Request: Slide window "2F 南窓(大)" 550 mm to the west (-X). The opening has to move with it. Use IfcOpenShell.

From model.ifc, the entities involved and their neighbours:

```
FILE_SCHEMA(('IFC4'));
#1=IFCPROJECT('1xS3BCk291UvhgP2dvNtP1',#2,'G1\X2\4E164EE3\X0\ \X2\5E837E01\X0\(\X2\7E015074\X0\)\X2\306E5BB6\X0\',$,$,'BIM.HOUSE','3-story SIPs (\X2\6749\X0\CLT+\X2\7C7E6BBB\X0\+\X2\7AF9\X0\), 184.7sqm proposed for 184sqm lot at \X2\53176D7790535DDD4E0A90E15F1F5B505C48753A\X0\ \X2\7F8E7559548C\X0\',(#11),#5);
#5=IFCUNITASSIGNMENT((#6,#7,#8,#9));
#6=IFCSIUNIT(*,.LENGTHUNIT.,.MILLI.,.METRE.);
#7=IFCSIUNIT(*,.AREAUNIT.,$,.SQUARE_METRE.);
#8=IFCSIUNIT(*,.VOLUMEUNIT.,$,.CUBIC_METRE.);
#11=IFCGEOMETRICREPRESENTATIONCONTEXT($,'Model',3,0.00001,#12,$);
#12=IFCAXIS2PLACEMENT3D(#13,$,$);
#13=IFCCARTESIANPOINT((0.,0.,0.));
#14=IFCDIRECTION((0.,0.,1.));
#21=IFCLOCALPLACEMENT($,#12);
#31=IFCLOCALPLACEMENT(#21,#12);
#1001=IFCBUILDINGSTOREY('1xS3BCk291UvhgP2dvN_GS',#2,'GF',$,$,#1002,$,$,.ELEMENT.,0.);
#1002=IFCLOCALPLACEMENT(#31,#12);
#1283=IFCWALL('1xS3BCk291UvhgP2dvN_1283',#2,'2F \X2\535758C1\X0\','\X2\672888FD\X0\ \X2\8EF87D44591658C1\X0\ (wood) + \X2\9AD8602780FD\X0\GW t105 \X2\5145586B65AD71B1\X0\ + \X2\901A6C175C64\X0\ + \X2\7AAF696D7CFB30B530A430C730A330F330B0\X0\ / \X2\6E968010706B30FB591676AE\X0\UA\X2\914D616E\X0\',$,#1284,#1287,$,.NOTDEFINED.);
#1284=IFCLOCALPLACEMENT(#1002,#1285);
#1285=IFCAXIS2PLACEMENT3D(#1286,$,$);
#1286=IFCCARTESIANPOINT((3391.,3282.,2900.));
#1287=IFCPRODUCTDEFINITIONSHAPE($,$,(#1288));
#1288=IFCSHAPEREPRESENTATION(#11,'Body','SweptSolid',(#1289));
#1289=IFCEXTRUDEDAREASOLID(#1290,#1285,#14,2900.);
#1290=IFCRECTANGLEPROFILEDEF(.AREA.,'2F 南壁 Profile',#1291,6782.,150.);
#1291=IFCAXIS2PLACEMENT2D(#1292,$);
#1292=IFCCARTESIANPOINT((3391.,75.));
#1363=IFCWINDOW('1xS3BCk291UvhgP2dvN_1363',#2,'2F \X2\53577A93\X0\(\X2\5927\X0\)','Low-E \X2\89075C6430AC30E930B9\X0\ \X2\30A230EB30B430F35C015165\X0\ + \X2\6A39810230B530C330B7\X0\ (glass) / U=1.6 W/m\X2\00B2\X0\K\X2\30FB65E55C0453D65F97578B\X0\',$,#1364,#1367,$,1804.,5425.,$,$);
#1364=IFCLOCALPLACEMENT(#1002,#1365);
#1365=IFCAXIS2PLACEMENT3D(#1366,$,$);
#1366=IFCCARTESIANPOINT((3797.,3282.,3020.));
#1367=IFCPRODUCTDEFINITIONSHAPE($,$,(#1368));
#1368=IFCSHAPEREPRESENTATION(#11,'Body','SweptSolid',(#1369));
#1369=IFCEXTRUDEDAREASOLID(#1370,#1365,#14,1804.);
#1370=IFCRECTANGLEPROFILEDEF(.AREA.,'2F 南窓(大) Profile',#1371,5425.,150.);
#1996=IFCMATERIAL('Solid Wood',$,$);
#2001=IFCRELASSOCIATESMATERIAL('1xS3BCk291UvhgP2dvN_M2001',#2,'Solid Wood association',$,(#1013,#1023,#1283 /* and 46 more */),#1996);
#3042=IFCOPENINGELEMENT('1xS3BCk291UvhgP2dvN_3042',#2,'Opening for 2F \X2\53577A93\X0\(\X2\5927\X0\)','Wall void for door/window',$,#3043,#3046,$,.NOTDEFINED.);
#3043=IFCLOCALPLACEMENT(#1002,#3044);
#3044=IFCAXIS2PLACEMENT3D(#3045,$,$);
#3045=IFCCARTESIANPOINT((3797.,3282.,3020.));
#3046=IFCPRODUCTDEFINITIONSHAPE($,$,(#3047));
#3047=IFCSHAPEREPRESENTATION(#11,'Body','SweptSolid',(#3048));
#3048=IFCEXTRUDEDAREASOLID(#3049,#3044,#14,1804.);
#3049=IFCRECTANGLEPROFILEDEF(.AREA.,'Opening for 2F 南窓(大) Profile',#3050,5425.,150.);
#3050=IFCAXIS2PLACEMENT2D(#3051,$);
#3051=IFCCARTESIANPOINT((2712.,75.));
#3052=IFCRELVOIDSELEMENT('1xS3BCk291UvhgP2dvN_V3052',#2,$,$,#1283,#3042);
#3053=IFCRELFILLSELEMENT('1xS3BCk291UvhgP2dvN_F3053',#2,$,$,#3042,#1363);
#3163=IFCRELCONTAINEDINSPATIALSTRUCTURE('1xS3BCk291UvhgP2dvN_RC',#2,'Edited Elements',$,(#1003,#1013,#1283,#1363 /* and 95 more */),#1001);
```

```python
import ifcopenshell
import ifcopenshell.api.geometry
import ifcopenshell.util.placement
import ifcopenshell.util.unit

model = ifcopenshell.open("model.ifc")
unit_scale = ifcopenshell.util.unit.calculate_unit_scale(model)

window = model.by_id(1363)
opening = window.FillsVoids[0].RelatingOpeningElement
wall = opening.VoidsElements[0].RelatingBuildingElement

wall_matrix = ifcopenshell.util.placement.get_local_placement(wall.ObjectPlacement)
shift = wall_matrix[:3, 0] * -0.55 / unit_scale
before = ifcopenshell.util.placement.get_local_placement(window.ObjectPlacement)[:3, 3].copy()

# The window is not placed relative to its opening, so move both.
for product in (opening, window):
    matrix = ifcopenshell.util.placement.get_local_placement(product.ObjectPlacement)
    matrix[:3, 3] += shift
    ifcopenshell.api.geometry.edit_object_placement(model, product=product, matrix=matrix, is_si=False)

after = ifcopenshell.util.placement.get_local_placement(window.ObjectPlacement)[:3, 3]
print("window moved by", (after - before).round(3) + 0.0)

model.write("model_edited.ifc")
```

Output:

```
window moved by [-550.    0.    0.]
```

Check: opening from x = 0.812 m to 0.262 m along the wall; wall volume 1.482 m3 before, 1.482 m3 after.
